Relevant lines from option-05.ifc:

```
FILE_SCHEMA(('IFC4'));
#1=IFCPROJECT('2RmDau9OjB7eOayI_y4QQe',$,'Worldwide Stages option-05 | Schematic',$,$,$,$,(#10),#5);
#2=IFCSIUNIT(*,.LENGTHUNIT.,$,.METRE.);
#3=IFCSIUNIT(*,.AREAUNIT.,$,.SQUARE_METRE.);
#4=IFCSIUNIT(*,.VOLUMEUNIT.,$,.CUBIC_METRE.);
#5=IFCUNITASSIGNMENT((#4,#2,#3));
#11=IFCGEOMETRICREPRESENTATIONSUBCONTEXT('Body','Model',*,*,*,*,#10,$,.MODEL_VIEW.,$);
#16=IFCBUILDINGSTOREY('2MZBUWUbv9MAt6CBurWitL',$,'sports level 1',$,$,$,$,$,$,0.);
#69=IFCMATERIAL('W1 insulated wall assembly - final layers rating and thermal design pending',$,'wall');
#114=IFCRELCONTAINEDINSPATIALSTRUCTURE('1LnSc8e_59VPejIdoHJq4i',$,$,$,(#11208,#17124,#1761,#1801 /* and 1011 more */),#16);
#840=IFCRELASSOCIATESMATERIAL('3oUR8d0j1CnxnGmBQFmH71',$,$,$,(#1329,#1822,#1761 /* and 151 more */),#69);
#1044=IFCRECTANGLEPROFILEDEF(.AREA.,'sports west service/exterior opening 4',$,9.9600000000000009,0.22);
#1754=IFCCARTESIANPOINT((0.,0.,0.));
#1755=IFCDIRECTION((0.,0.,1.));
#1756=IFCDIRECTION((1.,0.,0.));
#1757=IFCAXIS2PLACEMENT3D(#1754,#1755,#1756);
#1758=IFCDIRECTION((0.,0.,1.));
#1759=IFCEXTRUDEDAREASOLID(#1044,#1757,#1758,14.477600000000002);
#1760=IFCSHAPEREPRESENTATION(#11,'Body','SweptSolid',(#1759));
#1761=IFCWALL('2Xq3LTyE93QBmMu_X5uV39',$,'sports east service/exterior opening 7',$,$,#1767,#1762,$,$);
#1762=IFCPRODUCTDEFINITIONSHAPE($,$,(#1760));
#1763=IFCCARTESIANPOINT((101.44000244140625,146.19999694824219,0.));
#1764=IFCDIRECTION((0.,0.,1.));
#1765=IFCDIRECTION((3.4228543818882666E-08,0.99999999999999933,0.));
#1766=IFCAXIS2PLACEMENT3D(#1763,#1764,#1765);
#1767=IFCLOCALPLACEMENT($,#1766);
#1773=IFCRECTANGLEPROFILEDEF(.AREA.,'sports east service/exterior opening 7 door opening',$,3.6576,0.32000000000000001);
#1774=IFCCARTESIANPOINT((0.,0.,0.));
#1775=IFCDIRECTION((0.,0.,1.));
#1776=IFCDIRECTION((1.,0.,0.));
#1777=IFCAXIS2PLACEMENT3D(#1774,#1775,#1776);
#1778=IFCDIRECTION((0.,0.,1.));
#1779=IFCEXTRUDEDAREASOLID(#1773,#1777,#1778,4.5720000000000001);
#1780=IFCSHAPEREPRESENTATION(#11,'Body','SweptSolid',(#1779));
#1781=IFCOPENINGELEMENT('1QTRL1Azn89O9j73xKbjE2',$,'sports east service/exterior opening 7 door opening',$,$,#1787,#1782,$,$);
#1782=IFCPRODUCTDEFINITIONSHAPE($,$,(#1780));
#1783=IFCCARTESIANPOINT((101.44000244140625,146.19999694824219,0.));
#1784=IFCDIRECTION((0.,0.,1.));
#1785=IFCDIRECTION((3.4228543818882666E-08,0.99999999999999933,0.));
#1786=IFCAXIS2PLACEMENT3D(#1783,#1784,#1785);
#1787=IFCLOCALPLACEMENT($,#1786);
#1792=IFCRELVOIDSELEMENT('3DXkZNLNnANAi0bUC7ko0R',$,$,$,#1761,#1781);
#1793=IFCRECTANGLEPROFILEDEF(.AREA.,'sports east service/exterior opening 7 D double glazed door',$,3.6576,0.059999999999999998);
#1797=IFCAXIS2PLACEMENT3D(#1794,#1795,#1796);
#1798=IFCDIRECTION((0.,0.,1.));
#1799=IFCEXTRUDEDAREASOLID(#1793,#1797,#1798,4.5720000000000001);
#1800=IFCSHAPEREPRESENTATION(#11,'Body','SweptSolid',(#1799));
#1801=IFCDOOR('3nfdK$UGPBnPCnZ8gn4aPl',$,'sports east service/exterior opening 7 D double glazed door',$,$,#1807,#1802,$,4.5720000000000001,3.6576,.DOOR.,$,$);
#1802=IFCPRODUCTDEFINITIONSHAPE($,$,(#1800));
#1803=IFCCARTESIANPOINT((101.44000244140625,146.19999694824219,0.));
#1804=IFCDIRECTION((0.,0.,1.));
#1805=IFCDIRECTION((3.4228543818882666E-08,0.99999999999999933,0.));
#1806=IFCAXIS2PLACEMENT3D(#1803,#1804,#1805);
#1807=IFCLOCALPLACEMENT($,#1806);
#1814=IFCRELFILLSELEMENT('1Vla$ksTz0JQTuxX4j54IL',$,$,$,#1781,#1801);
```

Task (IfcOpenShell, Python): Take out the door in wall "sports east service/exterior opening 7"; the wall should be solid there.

```python
import ifcopenshell
import ifcopenshell.api.feature
import ifcopenshell.api.root
import ifcopenshell.geom
import ifcopenshell.util.shape

model = ifcopenshell.open("option-05.ifc")
settings = ifcopenshell.geom.settings()


def volume(element):
    """Net volume in cubic metres, openings subtracted."""
    shape = ifcopenshell.geom.create_shape(settings, element)
    return ifcopenshell.util.shape.get_volume(shape.geometry)


door = model.by_guid("3nfdK$UGPBnPCnZ8gn4aPl")
opening = door.FillsVoids[0].RelatingOpeningElement
wall = opening.VoidsElements[0].RelatingBuildingElement
before = volume(wall)

ifcopenshell.api.root.remove_product(model, product=door)
ifcopenshell.api.feature.remove_feature(model, feature=opening)

after = volume(wall)

print(f"wall volume {before:.3f} -> {after:.3f} m3")

model.write("option-05_v2.ifc")
```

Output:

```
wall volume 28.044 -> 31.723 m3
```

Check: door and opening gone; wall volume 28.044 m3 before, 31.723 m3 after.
